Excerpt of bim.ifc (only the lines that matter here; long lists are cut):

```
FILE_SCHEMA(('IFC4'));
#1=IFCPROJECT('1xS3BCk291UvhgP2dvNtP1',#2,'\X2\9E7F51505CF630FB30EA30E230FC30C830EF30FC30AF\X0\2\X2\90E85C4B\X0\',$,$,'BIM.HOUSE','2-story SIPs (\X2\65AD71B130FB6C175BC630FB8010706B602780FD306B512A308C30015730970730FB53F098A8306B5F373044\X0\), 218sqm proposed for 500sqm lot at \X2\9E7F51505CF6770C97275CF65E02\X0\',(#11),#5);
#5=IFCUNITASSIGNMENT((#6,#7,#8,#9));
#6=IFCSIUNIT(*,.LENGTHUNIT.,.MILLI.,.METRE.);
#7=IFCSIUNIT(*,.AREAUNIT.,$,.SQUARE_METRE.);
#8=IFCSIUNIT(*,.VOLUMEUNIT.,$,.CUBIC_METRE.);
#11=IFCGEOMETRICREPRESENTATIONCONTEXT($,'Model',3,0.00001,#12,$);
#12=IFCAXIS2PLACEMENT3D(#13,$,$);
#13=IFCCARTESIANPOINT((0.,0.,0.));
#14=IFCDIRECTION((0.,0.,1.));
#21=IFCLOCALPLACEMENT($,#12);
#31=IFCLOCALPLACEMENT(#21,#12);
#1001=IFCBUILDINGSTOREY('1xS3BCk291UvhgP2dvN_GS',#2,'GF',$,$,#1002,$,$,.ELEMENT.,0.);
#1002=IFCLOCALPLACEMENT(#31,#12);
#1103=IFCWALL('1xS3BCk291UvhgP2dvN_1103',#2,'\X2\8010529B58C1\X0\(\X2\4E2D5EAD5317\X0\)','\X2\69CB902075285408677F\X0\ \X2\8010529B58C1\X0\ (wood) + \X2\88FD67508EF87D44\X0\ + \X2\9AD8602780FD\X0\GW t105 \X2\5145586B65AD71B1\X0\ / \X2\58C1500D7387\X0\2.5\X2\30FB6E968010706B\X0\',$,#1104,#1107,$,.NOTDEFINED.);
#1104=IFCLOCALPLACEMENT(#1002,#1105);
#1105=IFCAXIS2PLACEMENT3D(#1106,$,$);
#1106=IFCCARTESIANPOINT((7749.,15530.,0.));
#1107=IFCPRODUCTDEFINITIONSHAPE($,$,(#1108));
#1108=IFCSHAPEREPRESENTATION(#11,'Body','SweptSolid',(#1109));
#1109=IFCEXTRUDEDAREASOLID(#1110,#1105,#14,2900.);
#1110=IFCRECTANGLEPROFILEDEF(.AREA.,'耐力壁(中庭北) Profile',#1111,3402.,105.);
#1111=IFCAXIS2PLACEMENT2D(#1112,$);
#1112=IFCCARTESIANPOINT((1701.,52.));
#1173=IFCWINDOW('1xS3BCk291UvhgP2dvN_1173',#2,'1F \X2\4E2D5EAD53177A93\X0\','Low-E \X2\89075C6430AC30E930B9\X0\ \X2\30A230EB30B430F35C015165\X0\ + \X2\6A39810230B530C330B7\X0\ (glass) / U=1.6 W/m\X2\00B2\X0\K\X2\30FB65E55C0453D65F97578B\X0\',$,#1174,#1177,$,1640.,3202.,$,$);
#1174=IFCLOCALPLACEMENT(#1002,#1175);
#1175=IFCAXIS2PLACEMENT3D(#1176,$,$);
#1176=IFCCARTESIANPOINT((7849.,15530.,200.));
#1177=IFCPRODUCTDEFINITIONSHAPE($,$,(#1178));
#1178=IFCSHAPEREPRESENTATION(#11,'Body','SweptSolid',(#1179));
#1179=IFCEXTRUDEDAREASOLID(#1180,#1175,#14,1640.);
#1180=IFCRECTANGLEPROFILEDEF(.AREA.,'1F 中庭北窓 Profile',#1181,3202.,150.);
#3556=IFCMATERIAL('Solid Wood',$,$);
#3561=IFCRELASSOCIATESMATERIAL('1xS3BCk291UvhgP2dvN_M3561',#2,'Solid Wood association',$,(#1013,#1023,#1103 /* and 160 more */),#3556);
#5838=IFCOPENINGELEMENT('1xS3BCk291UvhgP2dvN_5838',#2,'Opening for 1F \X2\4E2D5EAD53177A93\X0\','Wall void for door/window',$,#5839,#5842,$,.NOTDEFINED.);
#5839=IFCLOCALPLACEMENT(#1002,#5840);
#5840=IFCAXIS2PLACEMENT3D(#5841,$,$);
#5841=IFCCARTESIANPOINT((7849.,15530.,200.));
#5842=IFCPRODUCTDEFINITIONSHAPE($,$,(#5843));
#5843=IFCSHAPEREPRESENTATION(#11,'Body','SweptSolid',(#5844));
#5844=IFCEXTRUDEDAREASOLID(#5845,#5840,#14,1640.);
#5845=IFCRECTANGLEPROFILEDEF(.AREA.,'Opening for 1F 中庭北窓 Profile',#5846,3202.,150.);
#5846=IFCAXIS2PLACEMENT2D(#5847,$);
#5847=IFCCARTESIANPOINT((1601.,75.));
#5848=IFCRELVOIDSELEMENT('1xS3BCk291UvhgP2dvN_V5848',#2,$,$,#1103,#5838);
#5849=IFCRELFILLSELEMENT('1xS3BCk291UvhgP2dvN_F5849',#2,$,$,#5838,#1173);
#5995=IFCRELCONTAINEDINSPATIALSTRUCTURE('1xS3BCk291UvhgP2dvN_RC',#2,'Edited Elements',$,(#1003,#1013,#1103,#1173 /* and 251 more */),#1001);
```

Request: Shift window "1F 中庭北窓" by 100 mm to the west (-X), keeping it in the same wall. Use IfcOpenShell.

```python
import ifcopenshell
import ifcopenshell.api.geometry
import ifcopenshell.util.placement
import ifcopenshell.util.unit

model = ifcopenshell.open("bim.ifc")
unit_scale = ifcopenshell.util.unit.calculate_unit_scale(model)

window = model.by_id(1173)
opening = window.FillsVoids[0].RelatingOpeningElement
wall = opening.VoidsElements[0].RelatingBuildingElement

wall_matrix = ifcopenshell.util.placement.get_local_placement(wall.ObjectPlacement)
shift = wall_matrix[:3, 0] * -0.1 / unit_scale
before = ifcopenshell.util.placement.get_local_placement(window.ObjectPlacement)[:3, 3].copy()

# The window is not placed relative to its opening, so move both.
for product in (opening, window):
    matrix = ifcopenshell.util.placement.get_local_placement(product.ObjectPlacement)
    matrix[:3, 3] += shift
    ifcopenshell.api.geometry.edit_object_placement(model, product=product, matrix=matrix, is_si=False)

after = ifcopenshell.util.placement.get_local_placement(window.ObjectPlacement)[:3, 3]
print("window moved by", (after - before).round(3) + 0.0)

model.write("bim_v2.ifc")
```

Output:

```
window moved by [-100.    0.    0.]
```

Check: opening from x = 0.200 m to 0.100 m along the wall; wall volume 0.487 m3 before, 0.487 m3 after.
